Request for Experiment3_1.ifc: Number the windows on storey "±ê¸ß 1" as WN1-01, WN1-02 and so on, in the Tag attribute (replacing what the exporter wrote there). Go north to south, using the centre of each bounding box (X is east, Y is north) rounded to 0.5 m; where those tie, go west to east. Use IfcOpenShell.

First a look at what the model holds.

```python
import ifcopenshell
import ifcopenshell.util.element
import ifcopenshell.util.placement

model = ifcopenshell.open("Experiment3_1.ifc")
print(model.schema)
storey = next(s for s in model.by_type("IfcBuildingStorey") if s.Name == "±ê¸ß 1")
windows = [e for e in ifcopenshell.util.element.get_decomposition(storey) if e.is_a("IfcWindow")]
for e in sorted(windows, key=lambda e: e.id()):
    origin = ifcopenshell.util.placement.get_local_placement(e.ObjectPlacement)[:3, 3]
    print(e.id(), e.Tag, e.Name, origin.round(2) + 0.0, sep=" | ")
```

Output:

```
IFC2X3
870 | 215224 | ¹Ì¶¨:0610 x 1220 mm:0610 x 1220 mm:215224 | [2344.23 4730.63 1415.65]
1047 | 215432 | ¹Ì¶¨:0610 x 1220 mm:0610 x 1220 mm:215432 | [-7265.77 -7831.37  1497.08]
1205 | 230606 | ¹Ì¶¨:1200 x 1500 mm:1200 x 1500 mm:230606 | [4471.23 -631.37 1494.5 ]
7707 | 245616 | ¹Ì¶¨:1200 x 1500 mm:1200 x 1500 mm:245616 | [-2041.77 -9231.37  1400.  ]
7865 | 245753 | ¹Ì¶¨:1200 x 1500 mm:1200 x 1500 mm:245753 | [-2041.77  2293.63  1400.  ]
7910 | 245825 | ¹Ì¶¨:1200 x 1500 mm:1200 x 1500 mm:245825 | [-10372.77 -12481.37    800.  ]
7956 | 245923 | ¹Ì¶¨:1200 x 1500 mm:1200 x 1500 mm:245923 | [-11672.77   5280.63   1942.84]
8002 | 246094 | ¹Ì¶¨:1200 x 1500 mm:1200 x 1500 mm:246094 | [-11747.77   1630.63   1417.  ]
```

```python
import ifcopenshell
import ifcopenshell.geom
import ifcopenshell.util.element
import ifcopenshell.util.shape

model = ifcopenshell.open("Experiment3_1.ifc")
settings = ifcopenshell.geom.settings()
settings.set("use-world-coords", True)


def centre(element):
    shape = ifcopenshell.geom.create_shape(settings, element)
    return ifcopenshell.util.shape.get_bbox_centroid(shape.geometry)


storey = next(s for s in model.by_type("IfcBuildingStorey") if s.Name == "±ê¸ß 1")
windows = [e for e in ifcopenshell.util.element.get_decomposition(storey) if e.is_a("IfcWindow")]

# Insertion points can sit at a corner or the storey origin, so sort by the geometry (in metres).
centres = {e: centre(e) for e in windows}
windows.sort(key=lambda e: (-round(centres[e][1] / 0.5), centres[e][0]))

for i, e in enumerate(windows, start=1):
    number = f"WN1-{i:02d}"
    e.Tag = number
    print(e.id(), number)

model.write("Experiment3_1_edited.ifc")
```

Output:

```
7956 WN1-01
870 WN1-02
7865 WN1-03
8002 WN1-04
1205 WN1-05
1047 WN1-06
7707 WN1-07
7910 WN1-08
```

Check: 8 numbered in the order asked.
